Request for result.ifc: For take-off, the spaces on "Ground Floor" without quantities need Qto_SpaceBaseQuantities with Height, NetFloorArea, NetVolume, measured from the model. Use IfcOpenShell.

First a look at what the model holds.

```python
import ifcopenshell
import ifcopenshell.util.element
import ifcopenshell.util.unit

model = ifcopenshell.open("result.ifc")
print(model.schema)
for unit_type in ("LENGTHUNIT", "AREAUNIT", "VOLUMEUNIT"):
    print(unit_type, ifcopenshell.util.unit.calculate_unit_scale(model, unit_type))
storey = next(s for s in model.by_type("IfcBuildingStorey") if s.Name == "Ground Floor")
spaces = [e for e in ifcopenshell.util.element.get_decomposition(storey) if e.is_a("IfcSpace")]
for e in sorted(spaces, key=lambda e: e.id()):
    print(e.id(), e.is_a(), e.Name, list(ifcopenshell.util.element.get_psets(e, qtos_only=True)), sep=" | ")
```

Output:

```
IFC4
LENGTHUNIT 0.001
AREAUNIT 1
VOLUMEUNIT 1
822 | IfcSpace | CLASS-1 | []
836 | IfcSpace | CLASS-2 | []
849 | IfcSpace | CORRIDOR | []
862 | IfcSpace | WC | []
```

```python
import ifcopenshell
import ifcopenshell.api.pset
import ifcopenshell.geom
import ifcopenshell.util.element
import ifcopenshell.util.shape
import ifcopenshell.util.unit

model = ifcopenshell.open("result.ifc")
unit_scale = ifcopenshell.util.unit.calculate_unit_scale(model)
area_scale = ifcopenshell.util.unit.calculate_unit_scale(model, "AREAUNIT")
volume_scale = ifcopenshell.util.unit.calculate_unit_scale(model, "VOLUMEUNIT")
settings = ifcopenshell.geom.settings()

storey = next(s for s in model.by_type("IfcBuildingStorey") if s.Name == "Ground Floor")
spaces = [e for e in ifcopenshell.util.element.get_decomposition(storey) if e.is_a("IfcSpace")]

for e in sorted(spaces, key=lambda e: e.id()):
    if ifcopenshell.util.element.get_psets(e, qtos_only=True, should_inherit=False):
        continue
    # Geometry comes back in metres, in the element's own axes.
    shape = ifcopenshell.geom.create_shape(settings, e)
    values = {
        "Height": ifcopenshell.util.shape.get_z(shape.geometry) / unit_scale,
        "NetFloorArea": ifcopenshell.util.shape.get_footprint_area(shape.geometry) / area_scale,
        "NetVolume": ifcopenshell.util.shape.get_volume(shape.geometry) / volume_scale,
    }
    qto = ifcopenshell.api.pset.add_qto(model, product=e, name="Qto_SpaceBaseQuantities")
    ifcopenshell.api.pset.edit_qto(model, qto=qto, properties=values)
    print(e.id(), {k: round(v, 3) for k, v in values.items()})

model.write("result_v2.ifc")
```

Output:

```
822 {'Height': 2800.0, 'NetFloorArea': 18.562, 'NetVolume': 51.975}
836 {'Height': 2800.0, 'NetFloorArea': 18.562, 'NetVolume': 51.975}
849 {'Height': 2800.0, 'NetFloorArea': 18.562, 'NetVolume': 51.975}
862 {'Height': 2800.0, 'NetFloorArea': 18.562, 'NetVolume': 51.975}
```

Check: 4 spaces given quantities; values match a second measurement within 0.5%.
